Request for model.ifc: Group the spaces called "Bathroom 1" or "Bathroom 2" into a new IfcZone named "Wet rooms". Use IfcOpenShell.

First a look at what the model holds.

```python
import ifcopenshell

model = ifcopenshell.open("model.ifc")
print(model.schema)
seen = {}
for space in model.by_type("IfcSpace"):
    seen[space.LongName] = seen.get(space.LongName, 0) + 1
for name, count in sorted(seen.items(), key=str):
    print(count, "x", name)
print("zones:", [z.Name for z in model.by_type("IfcZone")][:20])
```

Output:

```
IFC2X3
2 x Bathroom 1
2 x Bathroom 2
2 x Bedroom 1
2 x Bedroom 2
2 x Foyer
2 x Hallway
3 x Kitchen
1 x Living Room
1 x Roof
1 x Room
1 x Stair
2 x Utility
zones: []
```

```python
import ifcopenshell
import ifcopenshell.api.group
import ifcopenshell.api.root

model = ifcopenshell.open("model.ifc")

names = {"Bathroom 1", "Bathroom 2"}
spaces = [s for s in model.by_type("IfcSpace") if s.LongName in names]

zone = ifcopenshell.api.root.create_entity(model, ifc_class="IfcZone", name="Wet rooms")
ifcopenshell.api.group.assign_group(model, products=spaces, group=zone)
print(len(spaces), "spaces in", zone.Name)

model.write("model_edited.ifc")
```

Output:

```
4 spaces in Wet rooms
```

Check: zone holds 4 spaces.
